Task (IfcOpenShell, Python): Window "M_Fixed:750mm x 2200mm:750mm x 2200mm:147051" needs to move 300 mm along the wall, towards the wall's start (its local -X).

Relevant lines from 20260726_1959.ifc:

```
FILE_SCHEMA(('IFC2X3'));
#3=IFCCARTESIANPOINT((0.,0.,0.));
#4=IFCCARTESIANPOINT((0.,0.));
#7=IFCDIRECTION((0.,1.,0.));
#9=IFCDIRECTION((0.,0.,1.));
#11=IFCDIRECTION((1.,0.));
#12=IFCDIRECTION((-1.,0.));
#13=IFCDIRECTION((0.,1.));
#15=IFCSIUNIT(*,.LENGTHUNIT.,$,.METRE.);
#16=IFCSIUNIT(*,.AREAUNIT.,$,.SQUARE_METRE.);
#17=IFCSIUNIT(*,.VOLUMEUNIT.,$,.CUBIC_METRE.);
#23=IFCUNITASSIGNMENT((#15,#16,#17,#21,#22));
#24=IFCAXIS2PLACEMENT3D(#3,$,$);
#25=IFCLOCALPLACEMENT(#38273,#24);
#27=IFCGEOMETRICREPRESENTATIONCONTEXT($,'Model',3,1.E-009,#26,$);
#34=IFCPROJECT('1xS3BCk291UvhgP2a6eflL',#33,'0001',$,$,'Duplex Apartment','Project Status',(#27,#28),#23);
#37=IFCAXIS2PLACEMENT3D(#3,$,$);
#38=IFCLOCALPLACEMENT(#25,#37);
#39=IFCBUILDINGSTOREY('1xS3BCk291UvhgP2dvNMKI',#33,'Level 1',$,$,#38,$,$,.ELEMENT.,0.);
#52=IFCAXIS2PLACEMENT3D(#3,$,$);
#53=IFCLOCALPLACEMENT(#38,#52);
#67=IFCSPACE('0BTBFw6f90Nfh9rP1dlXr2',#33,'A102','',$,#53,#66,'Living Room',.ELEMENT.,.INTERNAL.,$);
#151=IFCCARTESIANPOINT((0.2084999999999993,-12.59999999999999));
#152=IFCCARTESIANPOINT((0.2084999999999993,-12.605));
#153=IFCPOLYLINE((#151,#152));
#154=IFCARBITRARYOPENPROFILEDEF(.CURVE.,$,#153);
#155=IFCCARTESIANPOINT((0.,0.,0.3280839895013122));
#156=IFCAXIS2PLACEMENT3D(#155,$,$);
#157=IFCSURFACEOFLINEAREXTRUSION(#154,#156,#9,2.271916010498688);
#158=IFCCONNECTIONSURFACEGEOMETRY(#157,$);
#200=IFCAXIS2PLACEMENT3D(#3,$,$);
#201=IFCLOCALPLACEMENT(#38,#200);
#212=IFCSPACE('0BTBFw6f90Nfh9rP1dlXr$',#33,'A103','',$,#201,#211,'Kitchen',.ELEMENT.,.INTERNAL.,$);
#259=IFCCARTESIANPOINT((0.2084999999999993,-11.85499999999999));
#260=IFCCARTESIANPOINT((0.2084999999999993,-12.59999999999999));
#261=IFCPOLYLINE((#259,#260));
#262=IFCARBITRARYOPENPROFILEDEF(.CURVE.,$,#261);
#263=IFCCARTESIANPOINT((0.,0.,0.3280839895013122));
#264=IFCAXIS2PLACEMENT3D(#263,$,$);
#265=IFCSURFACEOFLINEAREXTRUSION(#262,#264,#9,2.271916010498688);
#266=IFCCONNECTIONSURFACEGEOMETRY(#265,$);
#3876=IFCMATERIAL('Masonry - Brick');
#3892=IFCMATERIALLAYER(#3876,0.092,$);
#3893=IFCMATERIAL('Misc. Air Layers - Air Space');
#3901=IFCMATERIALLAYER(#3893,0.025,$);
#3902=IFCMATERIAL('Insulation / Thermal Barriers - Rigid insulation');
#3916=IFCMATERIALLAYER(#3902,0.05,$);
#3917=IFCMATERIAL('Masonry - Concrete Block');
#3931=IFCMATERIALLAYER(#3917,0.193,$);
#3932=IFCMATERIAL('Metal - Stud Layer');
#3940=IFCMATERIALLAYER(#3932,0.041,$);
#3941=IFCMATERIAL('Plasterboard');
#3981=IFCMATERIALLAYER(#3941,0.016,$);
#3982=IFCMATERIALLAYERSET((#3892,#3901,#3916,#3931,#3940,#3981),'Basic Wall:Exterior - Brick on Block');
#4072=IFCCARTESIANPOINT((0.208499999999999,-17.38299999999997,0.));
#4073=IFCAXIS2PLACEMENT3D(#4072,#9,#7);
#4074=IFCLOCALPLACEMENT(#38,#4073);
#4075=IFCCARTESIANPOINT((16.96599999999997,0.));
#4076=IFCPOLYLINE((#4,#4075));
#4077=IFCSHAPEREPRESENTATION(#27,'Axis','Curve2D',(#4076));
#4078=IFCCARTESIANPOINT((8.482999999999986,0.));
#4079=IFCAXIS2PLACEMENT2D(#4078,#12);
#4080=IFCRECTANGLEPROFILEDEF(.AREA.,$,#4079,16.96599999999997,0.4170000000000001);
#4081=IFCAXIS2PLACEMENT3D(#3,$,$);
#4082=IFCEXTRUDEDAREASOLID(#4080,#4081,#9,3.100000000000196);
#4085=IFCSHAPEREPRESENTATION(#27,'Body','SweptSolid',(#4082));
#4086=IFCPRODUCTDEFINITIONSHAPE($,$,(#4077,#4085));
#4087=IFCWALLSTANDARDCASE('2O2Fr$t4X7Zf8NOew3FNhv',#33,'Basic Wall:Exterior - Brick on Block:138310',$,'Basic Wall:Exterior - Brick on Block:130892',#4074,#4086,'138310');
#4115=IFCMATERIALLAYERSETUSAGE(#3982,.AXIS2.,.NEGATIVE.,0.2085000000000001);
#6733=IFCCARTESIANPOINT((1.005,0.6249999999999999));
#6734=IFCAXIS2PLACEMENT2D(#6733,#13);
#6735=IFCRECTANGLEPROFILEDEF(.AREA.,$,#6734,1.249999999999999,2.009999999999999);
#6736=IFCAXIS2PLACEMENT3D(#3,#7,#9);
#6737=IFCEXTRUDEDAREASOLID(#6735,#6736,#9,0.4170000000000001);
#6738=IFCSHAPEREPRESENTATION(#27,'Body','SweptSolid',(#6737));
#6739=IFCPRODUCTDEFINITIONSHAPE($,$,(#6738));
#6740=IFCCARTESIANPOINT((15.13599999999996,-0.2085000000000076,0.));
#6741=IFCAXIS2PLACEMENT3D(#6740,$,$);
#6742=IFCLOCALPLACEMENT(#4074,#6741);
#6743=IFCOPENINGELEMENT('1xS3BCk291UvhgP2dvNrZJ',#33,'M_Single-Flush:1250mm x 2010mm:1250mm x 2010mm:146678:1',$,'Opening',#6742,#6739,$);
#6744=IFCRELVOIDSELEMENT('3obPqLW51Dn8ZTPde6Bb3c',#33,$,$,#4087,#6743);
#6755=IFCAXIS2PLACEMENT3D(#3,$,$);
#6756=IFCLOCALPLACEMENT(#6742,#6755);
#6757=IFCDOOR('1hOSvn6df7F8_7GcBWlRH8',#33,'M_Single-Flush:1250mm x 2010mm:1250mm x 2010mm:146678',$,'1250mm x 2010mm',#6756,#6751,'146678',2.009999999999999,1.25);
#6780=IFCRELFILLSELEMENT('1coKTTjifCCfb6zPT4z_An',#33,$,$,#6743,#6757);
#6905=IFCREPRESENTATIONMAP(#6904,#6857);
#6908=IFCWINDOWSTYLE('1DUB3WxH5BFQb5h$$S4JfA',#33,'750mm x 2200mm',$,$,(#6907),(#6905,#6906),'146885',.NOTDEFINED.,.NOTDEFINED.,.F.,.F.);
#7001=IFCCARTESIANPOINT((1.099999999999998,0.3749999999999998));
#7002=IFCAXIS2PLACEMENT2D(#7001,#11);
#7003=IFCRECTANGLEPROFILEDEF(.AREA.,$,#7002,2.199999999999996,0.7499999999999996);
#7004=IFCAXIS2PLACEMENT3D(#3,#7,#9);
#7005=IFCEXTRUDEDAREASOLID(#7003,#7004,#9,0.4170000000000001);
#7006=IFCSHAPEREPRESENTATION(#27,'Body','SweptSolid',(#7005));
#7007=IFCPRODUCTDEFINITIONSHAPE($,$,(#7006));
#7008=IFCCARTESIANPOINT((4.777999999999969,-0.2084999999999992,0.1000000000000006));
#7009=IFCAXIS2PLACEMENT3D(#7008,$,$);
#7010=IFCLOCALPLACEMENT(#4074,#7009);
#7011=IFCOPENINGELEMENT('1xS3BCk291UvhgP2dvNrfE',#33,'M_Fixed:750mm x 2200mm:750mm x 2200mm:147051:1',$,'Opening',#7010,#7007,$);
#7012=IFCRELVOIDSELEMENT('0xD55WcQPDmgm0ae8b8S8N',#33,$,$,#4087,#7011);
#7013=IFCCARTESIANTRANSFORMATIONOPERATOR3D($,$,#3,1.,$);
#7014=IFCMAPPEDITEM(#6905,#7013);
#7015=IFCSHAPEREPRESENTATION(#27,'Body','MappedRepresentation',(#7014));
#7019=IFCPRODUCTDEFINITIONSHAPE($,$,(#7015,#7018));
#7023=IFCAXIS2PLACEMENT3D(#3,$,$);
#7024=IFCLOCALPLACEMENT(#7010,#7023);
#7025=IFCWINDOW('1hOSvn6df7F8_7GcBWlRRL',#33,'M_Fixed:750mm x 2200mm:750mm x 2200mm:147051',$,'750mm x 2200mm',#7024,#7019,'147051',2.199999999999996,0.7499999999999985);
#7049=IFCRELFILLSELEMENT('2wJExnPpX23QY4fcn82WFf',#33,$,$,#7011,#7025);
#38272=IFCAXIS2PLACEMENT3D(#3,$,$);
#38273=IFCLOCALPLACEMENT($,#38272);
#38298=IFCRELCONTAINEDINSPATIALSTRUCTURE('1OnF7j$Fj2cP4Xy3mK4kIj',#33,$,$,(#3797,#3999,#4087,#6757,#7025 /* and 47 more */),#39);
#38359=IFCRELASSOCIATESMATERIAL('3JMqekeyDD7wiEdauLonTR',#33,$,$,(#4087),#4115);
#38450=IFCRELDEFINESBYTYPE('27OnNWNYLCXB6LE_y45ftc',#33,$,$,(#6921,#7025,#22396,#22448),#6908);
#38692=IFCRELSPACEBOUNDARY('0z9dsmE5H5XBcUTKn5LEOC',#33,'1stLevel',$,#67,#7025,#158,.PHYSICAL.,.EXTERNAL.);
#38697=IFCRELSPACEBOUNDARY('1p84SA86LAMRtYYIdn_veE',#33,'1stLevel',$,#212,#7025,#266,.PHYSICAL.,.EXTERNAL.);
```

```python
import numpy as np
import ifcopenshell
import ifcopenshell.api.geometry
import ifcopenshell.util.placement

model = ifcopenshell.open("20260726_1959.ifc")

window = model.by_id(7025)
opening = window.FillsVoids[0].RelatingOpeningElement
wall = opening.VoidsElements[0].RelatingBuildingElement

wall_matrix = ifcopenshell.util.placement.get_local_placement(wall.ObjectPlacement)
shift = wall_matrix[:3, 0] * -0.3
before = ifcopenshell.util.placement.get_local_placement(window.ObjectPlacement)[:3, 3].copy()

# The window is placed relative to its opening, so it follows when the opening moves.
matrix = ifcopenshell.util.placement.get_local_placement(opening.ObjectPlacement)
matrix[:3, 3] += shift
ifcopenshell.api.geometry.edit_object_placement(
    model, product=opening, matrix=matrix, is_si=False, should_transform_children=True
)

# Space boundary surfaces are stored in each space's coordinates; move them too.
for rel in window.ProvidesBoundaries:
    if not rel.ConnectionGeometry:
        continue
    surface = rel.ConnectionGeometry.SurfaceOnRelatingElement
    space_matrix = ifcopenshell.util.placement.get_local_placement(rel.RelatingSpace.ObjectPlacement)
    point = np.array(surface.Position.Location.Coordinates) + space_matrix[:3, :3].T @ shift
    surface.Position = model.createIfcAxis2Placement3D(
        model.createIfcCartesianPoint(point.tolist()), surface.Position.Axis, surface.Position.RefDirection
    )

after = ifcopenshell.util.placement.get_local_placement(window.ObjectPlacement)[:3, 3]
print("window moved by", (after - before).round(3) + 0.0)

model.write("20260726_1959_v2.ifc")
```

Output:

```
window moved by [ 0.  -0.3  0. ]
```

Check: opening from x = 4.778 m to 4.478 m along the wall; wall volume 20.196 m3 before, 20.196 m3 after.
